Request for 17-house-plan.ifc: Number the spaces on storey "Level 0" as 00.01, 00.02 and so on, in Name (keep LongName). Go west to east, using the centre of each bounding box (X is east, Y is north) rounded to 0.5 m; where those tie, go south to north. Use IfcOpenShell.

First a look at what the model holds.

```python
import ifcopenshell
import ifcopenshell.util.element
import ifcopenshell.util.placement

model = ifcopenshell.open("17-house-plan.ifc")
print(model.schema)
storey = next(s for s in model.by_type("IfcBuildingStorey") if s.Name == "Level 0")
spaces = [e for e in ifcopenshell.util.element.get_decomposition(storey) if e.is_a("IfcSpace")]
for e in sorted(spaces, key=lambda e: e.id()):
    origin = ifcopenshell.util.placement.get_local_placement(e.ObjectPlacement)[:3, 3]
    print(e.id(), e.Name, e.LongName, origin.round(2) + 0.0, sep=" | ")
```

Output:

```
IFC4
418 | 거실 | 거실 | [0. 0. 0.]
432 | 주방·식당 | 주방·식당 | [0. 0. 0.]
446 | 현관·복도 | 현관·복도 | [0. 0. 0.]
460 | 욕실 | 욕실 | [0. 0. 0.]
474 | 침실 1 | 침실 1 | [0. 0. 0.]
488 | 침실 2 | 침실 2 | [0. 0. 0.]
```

```python
import ifcopenshell
import ifcopenshell.geom
import ifcopenshell.util.element
import ifcopenshell.util.shape

model = ifcopenshell.open("17-house-plan.ifc")
settings = ifcopenshell.geom.settings()
settings.set("use-world-coords", True)


def centre(element):
    shape = ifcopenshell.geom.create_shape(settings, element)
    return ifcopenshell.util.shape.get_bbox_centroid(shape.geometry)


storey = next(s for s in model.by_type("IfcBuildingStorey") if s.Name == "Level 0")
spaces = [e for e in ifcopenshell.util.element.get_decomposition(storey) if e.is_a("IfcSpace")]

# Insertion points can sit at a corner or the storey origin, so sort by the geometry (in metres).
centres = {e: centre(e) for e in spaces}
spaces.sort(key=lambda e: (round(centres[e][0] / 0.5), centres[e][1]))

for i, e in enumerate(spaces, start=1):
    number = f"00.{i:02d}"
    e.Name = number
    print(e.id(), number)

model.write("17-house-plan_v2.ifc")
```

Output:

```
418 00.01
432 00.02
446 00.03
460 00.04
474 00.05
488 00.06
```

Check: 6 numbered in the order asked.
